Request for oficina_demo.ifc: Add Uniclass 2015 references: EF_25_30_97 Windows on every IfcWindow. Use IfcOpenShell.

First a look at what the model holds.

```python
import ifcopenshell

model = ifcopenshell.open("oficina_demo.ifc")
print(model.schema)
print("classifications:", [c.Name for c in model.by_type("IfcClassification")])
for ifc_class in ("IfcDoor", "IfcRoof", "IfcStair", "IfcWall", "IfcWindow"):
    print(ifc_class, len(model.by_type(ifc_class)))
```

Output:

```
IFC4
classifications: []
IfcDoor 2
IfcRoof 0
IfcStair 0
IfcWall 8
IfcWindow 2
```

```python
import ifcopenshell
import ifcopenshell.api.classification

model = ifcopenshell.open("oficina_demo.ifc")

system = ifcopenshell.api.classification.add_classification(model, classification="Uniclass 2015")

codes = {
    "IfcWindow": ("EF_25_30_97", "Windows"),
}
for ifc_class, (code, name) in codes.items():
    products = model.by_type(ifc_class)
    ifcopenshell.api.classification.add_reference(
        model, products=products, classification=system, identification=code, name=name
    )
    print(code, len(products))

model.write("oficina_demo_edited.ifc")
```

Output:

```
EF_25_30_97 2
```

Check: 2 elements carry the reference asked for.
